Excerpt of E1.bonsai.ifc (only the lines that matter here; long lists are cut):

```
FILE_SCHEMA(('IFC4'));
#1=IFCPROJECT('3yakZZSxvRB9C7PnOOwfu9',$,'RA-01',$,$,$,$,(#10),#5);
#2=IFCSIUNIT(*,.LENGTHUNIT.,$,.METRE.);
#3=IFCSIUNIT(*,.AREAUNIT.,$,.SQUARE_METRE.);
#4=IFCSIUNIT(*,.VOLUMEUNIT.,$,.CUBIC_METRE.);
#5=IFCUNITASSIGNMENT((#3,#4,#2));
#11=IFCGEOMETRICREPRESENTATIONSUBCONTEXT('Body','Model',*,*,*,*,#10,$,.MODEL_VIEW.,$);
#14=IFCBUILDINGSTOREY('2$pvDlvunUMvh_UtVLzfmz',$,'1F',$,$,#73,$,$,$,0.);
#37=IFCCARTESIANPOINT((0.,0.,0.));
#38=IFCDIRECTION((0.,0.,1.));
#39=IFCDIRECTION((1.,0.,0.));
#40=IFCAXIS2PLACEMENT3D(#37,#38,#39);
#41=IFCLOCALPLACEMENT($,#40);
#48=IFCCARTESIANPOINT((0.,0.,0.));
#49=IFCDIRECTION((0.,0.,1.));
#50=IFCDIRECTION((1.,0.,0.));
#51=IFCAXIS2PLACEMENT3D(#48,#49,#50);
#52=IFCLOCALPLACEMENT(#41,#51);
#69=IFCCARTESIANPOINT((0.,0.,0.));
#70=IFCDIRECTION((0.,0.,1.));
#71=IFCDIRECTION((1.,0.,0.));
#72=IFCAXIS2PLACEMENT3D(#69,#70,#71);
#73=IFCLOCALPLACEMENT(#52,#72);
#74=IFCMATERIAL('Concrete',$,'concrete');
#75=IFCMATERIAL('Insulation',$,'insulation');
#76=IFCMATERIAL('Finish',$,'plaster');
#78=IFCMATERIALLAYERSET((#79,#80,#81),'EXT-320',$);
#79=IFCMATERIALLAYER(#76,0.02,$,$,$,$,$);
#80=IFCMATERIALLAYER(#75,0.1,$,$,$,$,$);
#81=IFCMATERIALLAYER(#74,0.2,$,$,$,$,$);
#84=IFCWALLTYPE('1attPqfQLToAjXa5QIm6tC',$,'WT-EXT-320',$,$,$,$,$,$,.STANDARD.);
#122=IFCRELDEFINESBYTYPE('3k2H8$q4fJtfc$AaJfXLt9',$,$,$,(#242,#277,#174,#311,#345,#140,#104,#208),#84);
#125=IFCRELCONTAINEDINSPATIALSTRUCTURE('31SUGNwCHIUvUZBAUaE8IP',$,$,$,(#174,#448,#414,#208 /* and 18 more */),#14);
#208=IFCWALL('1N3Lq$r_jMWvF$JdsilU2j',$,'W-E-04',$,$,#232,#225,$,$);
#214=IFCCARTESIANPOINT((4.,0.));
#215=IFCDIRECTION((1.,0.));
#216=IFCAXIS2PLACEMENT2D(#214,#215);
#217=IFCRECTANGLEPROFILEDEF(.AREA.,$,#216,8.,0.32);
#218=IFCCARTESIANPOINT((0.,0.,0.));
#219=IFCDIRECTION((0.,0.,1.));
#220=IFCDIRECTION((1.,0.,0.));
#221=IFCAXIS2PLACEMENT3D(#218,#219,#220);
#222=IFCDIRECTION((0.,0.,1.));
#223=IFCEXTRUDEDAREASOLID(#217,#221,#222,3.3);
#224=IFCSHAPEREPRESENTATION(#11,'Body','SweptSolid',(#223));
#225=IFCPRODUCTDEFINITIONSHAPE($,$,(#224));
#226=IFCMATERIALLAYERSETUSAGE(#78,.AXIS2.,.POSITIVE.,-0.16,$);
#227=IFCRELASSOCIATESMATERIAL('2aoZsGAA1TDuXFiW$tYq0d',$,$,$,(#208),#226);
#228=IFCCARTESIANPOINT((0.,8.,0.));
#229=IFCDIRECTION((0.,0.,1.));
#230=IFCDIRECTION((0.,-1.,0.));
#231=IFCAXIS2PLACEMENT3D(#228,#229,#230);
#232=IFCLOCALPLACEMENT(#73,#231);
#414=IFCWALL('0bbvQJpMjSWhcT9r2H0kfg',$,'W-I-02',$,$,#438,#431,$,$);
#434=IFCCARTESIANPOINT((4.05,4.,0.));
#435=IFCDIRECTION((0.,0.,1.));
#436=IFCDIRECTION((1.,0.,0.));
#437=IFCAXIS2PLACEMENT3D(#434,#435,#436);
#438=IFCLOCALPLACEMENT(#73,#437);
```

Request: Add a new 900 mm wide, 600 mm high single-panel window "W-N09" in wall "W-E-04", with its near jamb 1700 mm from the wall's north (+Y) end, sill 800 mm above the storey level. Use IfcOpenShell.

```python
import numpy as np
import ifcopenshell
import ifcopenshell.api.feature
import ifcopenshell.api.geometry
import ifcopenshell.api.root
import ifcopenshell.api.spatial
import ifcopenshell.geom
import ifcopenshell.util.element
import ifcopenshell.util.placement
import ifcopenshell.util.representation
import ifcopenshell.util.shape
import ifcopenshell.util.unit

model = ifcopenshell.open("E1.bonsai.ifc")
unit_scale = ifcopenshell.util.unit.calculate_unit_scale(model)
settings = ifcopenshell.geom.settings()


def volume(element):
    """Net volume in cubic metres, openings subtracted."""
    shape = ifcopenshell.geom.create_shape(settings, element)
    return ifcopenshell.util.shape.get_volume(shape.geometry)


wall = model.by_guid("1N3Lq$r_jMWvF$JdsilU2j")
storey = ifcopenshell.util.element.get_container(wall, ifc_class="IfcBuildingStorey")
context = ifcopenshell.util.representation.get_context(model, "Model", "Body", "MODEL_VIEW")
before = volume(wall)

width, height, from_end, sill = 0.9, 0.6, 1.7, 0.8  # metres

# The wall runs along its own X axis, and the end named is its -X end.
wall_shape = ifcopenshell.geom.create_shape(settings, wall)
x, y, z = ifcopenshell.util.shape.get_vertices(wall_shape.geometry).T
start = x.min() + from_end
face, thickness = float(y.min()), float(y.max() - y.min())
wall_matrix = ifcopenshell.util.placement.get_local_placement(wall.ObjectPlacement)
level = ifcopenshell.util.placement.get_local_placement(storey.ObjectPlacement)[2, 3]


def in_wall(x, y):
    """Placement at x, y metres in the wall's axes, at sill height."""
    matrix = wall_matrix.copy()
    matrix[:, 3] = wall_matrix @ np.array([x / unit_scale, y / unit_scale, 0.0, 1.0])
    matrix[2, 3] = level + sill / unit_scale
    return matrix


# Opening: a box that overshoots both wall faces by 50 mm.
opening = ifcopenshell.api.root.create_entity(model, ifc_class="IfcOpeningElement", predefined_type="OPENING")
box = ifcopenshell.api.geometry.add_wall_representation(
    model, context=context, length=width, height=height, thickness=thickness + 0.1
)
ifcopenshell.api.geometry.assign_representation(model, product=opening, representation=box)
ifcopenshell.api.geometry.edit_object_placement(model, product=opening, matrix=in_wall(start, face - 0.05), is_si=False)
ifcopenshell.api.feature.add_feature(model, feature=opening, element=wall)

window = ifcopenshell.api.root.create_entity(model, ifc_class="IfcWindow", name="W-N09", predefined_type="WINDOW")
window.OverallWidth, window.OverallHeight = width / unit_scale, height / unit_scale
window.PartitioningType = "SINGLE_PANEL"
body = ifcopenshell.api.geometry.add_window_representation(
    model,
    context=context,
    overall_width=window.OverallWidth,
    overall_height=window.OverallHeight,
    partition_type="SINGLE_PANEL",
)
ifcopenshell.api.geometry.assign_representation(model, product=window, representation=body)
ifcopenshell.api.spatial.assign_container(model, products=[window], relating_structure=storey)
ifcopenshell.api.feature.add_filling(model, opening=opening, element=window)

# Centre the window in the wall's thickness.
ifcopenshell.api.geometry.edit_object_placement(model, product=window, matrix=in_wall(start, face), is_si=False)
window_shape = ifcopenshell.geom.create_shape(settings, window)
depth = ifcopenshell.util.shape.get_vertices(window_shape.geometry)[:, 1]
offset = face + thickness / 2 - (depth.min() + depth.max()) / 2
ifcopenshell.api.geometry.edit_object_placement(model, product=window, matrix=in_wall(start, offset), is_si=False)

after = volume(wall)

print(f"wall volume {before:.3f} -> {after:.3f} m3")

model.write("E1.bonsai_updated.ifc")
```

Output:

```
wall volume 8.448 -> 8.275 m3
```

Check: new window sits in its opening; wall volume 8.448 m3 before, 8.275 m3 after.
